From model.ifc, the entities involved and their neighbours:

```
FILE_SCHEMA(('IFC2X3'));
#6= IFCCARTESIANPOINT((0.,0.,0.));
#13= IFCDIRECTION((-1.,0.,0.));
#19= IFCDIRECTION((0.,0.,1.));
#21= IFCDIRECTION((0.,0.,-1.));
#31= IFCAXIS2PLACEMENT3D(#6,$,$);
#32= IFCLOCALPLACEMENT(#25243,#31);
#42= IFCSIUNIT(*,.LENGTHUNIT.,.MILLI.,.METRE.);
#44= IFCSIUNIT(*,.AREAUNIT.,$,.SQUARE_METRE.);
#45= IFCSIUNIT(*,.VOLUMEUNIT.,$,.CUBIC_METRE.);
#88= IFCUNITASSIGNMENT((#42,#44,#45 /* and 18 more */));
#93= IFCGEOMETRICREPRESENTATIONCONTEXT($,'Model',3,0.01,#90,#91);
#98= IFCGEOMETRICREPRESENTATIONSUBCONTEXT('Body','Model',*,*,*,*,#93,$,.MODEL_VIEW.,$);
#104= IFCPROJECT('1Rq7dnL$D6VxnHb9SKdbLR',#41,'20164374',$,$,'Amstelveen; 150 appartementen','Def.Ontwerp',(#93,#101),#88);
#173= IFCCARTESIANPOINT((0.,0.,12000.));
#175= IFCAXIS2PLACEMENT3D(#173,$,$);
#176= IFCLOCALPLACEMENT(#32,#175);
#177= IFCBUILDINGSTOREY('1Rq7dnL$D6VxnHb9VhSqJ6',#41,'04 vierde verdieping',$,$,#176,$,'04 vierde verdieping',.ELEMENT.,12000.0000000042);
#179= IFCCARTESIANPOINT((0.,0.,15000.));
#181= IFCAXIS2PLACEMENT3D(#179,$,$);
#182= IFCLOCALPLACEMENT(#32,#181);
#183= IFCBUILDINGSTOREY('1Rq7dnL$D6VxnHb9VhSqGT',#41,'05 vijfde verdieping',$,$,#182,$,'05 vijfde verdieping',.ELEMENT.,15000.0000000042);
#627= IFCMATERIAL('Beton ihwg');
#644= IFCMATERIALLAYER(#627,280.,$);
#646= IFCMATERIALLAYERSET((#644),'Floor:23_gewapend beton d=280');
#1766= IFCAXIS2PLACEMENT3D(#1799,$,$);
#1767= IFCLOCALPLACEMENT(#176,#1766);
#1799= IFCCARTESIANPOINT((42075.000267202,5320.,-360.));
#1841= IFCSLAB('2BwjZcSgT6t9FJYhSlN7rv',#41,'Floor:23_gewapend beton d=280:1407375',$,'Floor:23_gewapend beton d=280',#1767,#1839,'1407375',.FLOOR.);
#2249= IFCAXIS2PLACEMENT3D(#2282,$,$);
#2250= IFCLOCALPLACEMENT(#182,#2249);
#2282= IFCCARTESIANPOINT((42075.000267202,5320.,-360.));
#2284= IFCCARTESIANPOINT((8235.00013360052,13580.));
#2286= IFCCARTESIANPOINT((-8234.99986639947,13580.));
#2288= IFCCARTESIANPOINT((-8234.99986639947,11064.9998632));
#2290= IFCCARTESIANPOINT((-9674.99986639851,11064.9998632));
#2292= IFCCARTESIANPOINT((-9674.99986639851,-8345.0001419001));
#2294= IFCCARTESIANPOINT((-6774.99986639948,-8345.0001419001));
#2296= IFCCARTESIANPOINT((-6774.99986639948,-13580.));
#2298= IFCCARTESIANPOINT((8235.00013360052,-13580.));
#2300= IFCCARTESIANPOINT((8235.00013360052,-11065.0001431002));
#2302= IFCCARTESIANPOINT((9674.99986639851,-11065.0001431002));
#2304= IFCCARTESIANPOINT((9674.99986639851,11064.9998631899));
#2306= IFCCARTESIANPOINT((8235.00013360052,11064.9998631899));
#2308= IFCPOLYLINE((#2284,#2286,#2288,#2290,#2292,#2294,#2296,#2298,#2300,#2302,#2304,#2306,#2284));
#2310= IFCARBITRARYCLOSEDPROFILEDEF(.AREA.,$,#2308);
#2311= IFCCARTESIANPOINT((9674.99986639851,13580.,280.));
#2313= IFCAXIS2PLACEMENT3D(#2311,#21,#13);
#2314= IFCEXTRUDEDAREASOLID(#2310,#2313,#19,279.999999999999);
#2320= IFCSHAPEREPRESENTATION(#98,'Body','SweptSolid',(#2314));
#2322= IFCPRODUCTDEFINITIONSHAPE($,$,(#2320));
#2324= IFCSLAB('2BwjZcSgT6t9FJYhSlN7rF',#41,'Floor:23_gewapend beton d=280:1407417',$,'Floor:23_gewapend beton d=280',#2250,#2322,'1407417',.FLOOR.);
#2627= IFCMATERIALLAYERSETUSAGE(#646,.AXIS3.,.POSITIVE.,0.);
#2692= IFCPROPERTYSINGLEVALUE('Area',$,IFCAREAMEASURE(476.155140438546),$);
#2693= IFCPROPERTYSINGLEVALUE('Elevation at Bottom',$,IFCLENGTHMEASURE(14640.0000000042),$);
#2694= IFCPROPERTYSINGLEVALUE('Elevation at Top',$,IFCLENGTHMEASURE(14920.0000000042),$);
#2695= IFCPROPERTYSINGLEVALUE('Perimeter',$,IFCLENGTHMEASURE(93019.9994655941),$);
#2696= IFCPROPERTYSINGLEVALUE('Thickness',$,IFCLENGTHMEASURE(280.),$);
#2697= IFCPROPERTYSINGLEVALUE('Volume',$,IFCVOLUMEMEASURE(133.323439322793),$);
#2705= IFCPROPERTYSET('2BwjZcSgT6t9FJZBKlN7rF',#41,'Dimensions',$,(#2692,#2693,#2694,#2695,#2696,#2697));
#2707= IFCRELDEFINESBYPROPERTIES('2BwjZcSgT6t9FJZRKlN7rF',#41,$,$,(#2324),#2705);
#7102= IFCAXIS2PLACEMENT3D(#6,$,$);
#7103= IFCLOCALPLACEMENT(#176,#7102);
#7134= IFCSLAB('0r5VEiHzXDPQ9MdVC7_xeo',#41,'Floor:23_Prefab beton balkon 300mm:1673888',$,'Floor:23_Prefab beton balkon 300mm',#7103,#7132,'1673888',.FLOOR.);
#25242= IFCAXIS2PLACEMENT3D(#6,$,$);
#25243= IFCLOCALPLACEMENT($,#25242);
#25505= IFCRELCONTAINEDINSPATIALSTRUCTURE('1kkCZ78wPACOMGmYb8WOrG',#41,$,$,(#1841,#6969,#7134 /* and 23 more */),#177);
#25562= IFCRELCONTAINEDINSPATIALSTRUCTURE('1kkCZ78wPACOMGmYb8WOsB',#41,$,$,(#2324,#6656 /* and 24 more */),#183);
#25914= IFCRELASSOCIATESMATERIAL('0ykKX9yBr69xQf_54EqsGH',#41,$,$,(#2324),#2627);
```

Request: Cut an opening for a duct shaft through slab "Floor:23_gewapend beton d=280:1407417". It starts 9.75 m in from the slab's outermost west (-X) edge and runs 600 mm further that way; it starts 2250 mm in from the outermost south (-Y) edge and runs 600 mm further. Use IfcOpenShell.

```python
import numpy as np
import ifcopenshell
import ifcopenshell.api.feature
import ifcopenshell.api.geometry
import ifcopenshell.api.pset
import ifcopenshell.api.root
import ifcopenshell.geom
import ifcopenshell.util.element
import ifcopenshell.util.placement
import ifcopenshell.util.representation
import ifcopenshell.util.shape
import ifcopenshell.util.unit

model = ifcopenshell.open("model.ifc")
unit_scale = ifcopenshell.util.unit.calculate_unit_scale(model)
area_scale = ifcopenshell.util.unit.calculate_unit_scale(model, "AREAUNIT")
volume_scale = ifcopenshell.util.unit.calculate_unit_scale(model, "VOLUMEUNIT")
settings = ifcopenshell.geom.settings()


def volume(element):
    """Net volume in cubic metres, openings subtracted."""
    shape = ifcopenshell.geom.create_shape(settings, element)
    return ifcopenshell.util.shape.get_volume(shape.geometry)


slab = model.by_guid("2BwjZcSgT6t9FJYhSlN7rF")
before = volume(slab)

# Extent in the slab's own axes, in metres. The edges named are its -X and -Y sides.
slab_shape = ifcopenshell.geom.create_shape(settings, slab)
vertices = ifcopenshell.util.shape.get_vertices(slab_shape.geometry)
x_min, y_min, bottom = vertices.min(axis=0)
top = vertices[:, 2].max()

opening = ifcopenshell.api.root.create_entity(model, ifc_class="IfcOpeningElement", name="Duct shaft opening")
context = ifcopenshell.util.representation.get_context(model, "Model", "Body", "MODEL_VIEW")
width, depth = 0.6, 0.6
outline = [(0.0, 0.0), (width, 0.0), (width, depth), (0.0, depth), (0.0, 0.0)]
# Overshoot both faces by 50 mm so the cut is clean.
shape = ifcopenshell.api.geometry.add_slab_representation(
    model, context=context, depth=top - bottom + 0.1, polyline=outline
)
ifcopenshell.api.geometry.assign_representation(model, product=opening, representation=shape)

matrix = ifcopenshell.util.placement.get_local_placement(slab.ObjectPlacement)
matrix[:, 3] = matrix @ np.append(np.array([x_min + 9.75, y_min + 2.25, bottom - 0.05]) / unit_scale, 1.0)
ifcopenshell.api.geometry.edit_object_placement(model, product=opening, matrix=matrix, is_si=False)
ifcopenshell.api.feature.add_feature(model, feature=opening, element=slab)

after = volume(slab)

# Update the slab's stored quantities.
pset = model.by_id(ifcopenshell.util.element.get_pset(slab, "Dimensions", should_inherit=False)["id"])
ifcopenshell.api.pset.edit_pset(model, pset=pset, properties={
    "Area": model.create_entity("IfcAreaMeasure", after / (top - bottom) / area_scale),
    "Volume": model.create_entity("IfcVolumeMeasure", after / volume_scale),
})

print(f"slab volume {before:.3f} -> {after:.3f} m3")

model.write("model_edited.ifc")
```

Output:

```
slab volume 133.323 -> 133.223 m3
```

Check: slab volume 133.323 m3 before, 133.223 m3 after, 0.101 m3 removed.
